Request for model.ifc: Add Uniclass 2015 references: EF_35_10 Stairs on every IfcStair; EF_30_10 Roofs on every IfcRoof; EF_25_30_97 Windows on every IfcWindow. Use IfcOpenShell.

First a look at what the model holds.

```python
import ifcopenshell

model = ifcopenshell.open("model.ifc")
print(model.schema)
print("classifications:", [c.Name for c in model.by_type("IfcClassification")])
for ifc_class in ("IfcDoor", "IfcRoof", "IfcStair", "IfcWall", "IfcWindow"):
    print(ifc_class, len(model.by_type(ifc_class)))
```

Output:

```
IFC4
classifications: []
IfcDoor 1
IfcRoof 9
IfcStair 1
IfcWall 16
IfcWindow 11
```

```python
import ifcopenshell
import ifcopenshell.api.classification

model = ifcopenshell.open("model.ifc")

system = ifcopenshell.api.classification.add_classification(model, classification="Uniclass 2015")

codes = {
    "IfcStair": ("EF_35_10", "Stairs"),
    "IfcRoof": ("EF_30_10", "Roofs"),
    "IfcWindow": ("EF_25_30_97", "Windows"),
}
for ifc_class, (code, name) in codes.items():
    products = model.by_type(ifc_class)
    ifcopenshell.api.classification.add_reference(
        model, products=products, classification=system, identification=code, name=name
    )
    print(code, len(products))

model.write("model_edited.ifc")
```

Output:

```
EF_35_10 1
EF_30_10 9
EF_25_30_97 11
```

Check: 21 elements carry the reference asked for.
